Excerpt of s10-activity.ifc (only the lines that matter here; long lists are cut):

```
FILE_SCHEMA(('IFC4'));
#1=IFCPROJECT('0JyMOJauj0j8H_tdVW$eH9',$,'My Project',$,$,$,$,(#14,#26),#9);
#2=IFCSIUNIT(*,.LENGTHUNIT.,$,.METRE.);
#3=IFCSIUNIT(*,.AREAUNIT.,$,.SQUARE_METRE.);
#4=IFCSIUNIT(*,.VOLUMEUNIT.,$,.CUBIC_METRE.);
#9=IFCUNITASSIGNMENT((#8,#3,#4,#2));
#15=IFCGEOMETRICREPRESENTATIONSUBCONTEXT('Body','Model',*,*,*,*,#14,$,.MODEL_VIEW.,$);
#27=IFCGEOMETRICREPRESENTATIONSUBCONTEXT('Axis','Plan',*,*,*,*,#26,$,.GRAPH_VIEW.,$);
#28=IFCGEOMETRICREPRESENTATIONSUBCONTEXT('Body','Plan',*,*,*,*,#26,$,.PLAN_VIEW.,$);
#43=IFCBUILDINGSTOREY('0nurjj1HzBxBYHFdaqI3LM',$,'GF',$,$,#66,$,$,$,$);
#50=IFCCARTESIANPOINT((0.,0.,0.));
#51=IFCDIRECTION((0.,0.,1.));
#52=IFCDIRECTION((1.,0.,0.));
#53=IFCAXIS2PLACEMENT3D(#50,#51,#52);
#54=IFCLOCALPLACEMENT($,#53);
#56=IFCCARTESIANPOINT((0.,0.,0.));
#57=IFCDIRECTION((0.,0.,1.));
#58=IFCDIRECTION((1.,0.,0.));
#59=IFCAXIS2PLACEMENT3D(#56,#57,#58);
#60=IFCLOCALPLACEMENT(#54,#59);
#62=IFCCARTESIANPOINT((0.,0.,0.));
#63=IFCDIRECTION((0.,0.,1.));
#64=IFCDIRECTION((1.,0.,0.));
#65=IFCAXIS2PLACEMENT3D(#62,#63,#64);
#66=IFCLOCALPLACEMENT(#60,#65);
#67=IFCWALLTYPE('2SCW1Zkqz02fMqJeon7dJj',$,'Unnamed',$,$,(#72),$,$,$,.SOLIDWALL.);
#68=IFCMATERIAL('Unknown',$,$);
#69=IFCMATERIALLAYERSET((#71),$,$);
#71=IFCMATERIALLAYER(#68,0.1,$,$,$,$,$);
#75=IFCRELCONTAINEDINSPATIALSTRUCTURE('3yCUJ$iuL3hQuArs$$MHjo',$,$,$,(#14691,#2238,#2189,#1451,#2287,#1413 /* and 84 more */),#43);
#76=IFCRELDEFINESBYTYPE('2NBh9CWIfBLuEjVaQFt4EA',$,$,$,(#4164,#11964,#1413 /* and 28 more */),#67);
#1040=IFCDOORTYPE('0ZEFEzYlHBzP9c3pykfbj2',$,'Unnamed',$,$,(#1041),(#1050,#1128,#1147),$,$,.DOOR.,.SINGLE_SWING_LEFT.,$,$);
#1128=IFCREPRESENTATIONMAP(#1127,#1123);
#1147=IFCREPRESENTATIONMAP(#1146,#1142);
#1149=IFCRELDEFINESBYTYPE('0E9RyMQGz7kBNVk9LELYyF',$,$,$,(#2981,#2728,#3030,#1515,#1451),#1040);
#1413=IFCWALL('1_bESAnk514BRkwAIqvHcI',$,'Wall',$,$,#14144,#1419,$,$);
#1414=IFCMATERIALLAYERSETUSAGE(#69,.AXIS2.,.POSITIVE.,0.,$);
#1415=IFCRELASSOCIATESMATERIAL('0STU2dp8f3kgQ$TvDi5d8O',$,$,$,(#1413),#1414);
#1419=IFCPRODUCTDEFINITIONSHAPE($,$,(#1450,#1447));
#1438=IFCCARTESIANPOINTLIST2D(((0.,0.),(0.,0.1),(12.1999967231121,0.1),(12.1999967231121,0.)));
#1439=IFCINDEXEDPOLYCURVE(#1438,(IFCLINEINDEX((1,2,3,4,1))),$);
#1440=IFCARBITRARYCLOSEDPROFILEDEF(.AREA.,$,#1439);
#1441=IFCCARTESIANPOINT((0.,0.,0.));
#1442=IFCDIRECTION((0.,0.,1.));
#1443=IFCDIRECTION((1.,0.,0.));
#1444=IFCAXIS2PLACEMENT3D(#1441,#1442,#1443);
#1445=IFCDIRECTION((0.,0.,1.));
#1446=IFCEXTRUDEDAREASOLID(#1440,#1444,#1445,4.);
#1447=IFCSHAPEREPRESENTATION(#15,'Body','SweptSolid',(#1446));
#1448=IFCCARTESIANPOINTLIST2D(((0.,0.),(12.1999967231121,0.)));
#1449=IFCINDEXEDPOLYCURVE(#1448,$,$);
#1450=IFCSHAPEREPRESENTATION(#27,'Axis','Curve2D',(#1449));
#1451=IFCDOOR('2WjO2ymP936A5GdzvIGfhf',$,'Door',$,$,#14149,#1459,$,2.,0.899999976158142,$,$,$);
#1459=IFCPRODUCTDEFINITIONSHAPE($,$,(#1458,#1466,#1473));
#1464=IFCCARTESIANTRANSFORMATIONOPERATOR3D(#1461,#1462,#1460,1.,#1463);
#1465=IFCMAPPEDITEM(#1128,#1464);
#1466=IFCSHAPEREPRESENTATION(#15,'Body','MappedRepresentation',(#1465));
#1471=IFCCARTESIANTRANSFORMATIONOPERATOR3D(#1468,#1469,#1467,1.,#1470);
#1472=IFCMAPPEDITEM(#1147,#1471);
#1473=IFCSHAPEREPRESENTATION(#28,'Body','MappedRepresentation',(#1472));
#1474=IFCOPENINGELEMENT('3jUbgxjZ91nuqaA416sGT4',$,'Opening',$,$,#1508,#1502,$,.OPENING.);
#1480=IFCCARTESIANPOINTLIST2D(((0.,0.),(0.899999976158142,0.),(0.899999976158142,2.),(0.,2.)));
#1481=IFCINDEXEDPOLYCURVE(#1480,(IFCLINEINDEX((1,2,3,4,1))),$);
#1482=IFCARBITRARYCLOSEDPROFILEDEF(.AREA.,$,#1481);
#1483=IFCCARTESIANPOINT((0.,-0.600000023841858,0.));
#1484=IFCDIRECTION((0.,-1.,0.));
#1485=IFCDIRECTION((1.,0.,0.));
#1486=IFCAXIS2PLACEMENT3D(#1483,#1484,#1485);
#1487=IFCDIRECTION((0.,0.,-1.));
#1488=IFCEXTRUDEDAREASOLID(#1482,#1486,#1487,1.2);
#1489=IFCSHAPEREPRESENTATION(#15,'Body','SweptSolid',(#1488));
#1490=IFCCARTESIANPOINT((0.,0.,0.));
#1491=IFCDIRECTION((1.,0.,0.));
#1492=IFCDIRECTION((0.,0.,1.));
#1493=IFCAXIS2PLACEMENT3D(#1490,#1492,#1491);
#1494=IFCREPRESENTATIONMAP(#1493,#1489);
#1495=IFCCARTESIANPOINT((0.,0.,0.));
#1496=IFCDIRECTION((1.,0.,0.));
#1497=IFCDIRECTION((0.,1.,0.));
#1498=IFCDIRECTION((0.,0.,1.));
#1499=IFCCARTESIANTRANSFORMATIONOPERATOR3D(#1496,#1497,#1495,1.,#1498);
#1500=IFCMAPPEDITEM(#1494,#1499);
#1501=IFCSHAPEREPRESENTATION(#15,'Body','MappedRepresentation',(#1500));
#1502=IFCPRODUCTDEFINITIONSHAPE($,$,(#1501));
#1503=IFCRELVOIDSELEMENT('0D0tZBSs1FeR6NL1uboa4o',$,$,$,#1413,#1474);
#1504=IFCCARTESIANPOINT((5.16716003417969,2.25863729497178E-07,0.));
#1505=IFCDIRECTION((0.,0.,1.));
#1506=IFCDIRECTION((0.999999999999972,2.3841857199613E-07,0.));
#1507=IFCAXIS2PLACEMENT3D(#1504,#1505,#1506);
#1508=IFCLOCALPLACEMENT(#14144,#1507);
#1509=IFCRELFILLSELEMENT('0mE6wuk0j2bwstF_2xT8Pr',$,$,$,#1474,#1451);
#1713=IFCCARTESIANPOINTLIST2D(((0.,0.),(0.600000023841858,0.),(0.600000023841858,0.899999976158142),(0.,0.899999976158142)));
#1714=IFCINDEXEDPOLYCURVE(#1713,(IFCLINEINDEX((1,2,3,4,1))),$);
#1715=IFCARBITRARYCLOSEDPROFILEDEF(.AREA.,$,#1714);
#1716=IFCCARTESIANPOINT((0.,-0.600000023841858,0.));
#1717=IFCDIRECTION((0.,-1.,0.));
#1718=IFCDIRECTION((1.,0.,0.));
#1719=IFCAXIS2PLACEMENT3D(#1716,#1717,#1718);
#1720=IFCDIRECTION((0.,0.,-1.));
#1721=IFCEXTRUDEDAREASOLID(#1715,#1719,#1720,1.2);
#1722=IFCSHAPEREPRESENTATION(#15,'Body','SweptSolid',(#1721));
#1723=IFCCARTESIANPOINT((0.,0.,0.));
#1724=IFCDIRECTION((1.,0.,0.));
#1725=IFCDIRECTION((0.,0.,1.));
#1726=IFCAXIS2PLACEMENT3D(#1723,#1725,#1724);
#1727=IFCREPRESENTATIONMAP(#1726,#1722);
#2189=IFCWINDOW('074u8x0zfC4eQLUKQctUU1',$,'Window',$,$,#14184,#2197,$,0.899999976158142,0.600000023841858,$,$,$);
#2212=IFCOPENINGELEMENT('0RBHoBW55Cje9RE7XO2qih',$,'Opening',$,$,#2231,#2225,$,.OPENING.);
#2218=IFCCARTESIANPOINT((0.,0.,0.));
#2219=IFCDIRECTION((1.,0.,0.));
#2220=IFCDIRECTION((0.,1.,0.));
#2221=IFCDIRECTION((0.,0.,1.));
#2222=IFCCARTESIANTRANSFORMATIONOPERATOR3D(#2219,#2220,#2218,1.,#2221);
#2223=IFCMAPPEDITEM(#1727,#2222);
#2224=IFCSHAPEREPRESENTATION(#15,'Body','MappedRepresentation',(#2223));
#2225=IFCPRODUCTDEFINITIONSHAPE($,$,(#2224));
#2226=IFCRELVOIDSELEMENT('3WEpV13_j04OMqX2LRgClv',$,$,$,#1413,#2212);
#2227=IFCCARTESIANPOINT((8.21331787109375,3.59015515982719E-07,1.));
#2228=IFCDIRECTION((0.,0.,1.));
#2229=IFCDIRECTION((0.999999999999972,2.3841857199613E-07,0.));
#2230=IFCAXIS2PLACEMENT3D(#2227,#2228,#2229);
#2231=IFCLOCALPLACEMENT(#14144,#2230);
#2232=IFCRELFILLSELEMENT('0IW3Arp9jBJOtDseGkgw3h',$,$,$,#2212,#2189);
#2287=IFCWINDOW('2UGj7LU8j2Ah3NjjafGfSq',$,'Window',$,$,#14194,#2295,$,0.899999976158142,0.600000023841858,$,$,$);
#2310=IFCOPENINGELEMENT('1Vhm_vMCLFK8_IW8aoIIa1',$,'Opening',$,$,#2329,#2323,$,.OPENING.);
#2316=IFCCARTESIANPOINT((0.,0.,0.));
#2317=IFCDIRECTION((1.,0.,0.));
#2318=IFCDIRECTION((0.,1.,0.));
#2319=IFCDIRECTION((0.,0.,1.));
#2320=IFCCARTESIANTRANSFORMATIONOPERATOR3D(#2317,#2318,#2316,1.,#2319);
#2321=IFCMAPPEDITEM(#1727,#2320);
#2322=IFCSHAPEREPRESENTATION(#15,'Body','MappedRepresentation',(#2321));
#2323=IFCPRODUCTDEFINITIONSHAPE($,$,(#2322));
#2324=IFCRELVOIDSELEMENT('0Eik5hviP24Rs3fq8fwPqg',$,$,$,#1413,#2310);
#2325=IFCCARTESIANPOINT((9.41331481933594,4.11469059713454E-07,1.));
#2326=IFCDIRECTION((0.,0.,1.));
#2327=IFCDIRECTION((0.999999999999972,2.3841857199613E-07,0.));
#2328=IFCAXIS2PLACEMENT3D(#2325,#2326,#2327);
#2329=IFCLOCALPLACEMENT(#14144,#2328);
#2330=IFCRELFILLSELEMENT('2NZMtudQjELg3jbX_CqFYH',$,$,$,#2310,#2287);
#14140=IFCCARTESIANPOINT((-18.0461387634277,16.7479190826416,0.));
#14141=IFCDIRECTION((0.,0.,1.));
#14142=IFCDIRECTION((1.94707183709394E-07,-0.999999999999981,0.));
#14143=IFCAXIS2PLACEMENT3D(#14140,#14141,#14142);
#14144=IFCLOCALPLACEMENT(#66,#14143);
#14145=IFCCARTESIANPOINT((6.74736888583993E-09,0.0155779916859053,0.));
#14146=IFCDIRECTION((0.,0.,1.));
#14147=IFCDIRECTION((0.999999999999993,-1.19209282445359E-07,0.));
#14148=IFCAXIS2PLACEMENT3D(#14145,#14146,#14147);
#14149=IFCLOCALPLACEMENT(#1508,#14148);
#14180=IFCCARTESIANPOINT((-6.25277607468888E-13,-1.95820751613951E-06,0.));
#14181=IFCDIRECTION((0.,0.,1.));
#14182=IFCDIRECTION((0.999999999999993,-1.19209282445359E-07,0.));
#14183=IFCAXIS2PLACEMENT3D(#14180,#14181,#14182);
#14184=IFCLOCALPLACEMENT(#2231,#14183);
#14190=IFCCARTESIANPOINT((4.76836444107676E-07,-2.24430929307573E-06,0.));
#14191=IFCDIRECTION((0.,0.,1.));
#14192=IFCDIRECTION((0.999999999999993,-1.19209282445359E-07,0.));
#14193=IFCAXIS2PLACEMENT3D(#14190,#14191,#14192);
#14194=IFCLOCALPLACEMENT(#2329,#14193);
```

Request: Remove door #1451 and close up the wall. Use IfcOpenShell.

```python
import ifcopenshell
import ifcopenshell.api.feature
import ifcopenshell.api.root
import ifcopenshell.geom
import ifcopenshell.util.shape

model = ifcopenshell.open("s10-activity.ifc")
settings = ifcopenshell.geom.settings()


def volume(element):
    """Net volume in cubic metres, openings subtracted."""
    shape = ifcopenshell.geom.create_shape(settings, element)
    return ifcopenshell.util.shape.get_volume(shape.geometry)


door = model.by_guid("2WjO2ymP936A5GdzvIGfhf")
opening = door.FillsVoids[0].RelatingOpeningElement
wall = opening.VoidsElements[0].RelatingBuildingElement
before = volume(wall)

ifcopenshell.api.root.remove_product(model, product=door)
ifcopenshell.api.feature.remove_feature(model, feature=opening)

after = volume(wall)

print(f"wall volume {before:.3f} -> {after:.3f} m3")

model.write("s10-activity_v2.ifc")
```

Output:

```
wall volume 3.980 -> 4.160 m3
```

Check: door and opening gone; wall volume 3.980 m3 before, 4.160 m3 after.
